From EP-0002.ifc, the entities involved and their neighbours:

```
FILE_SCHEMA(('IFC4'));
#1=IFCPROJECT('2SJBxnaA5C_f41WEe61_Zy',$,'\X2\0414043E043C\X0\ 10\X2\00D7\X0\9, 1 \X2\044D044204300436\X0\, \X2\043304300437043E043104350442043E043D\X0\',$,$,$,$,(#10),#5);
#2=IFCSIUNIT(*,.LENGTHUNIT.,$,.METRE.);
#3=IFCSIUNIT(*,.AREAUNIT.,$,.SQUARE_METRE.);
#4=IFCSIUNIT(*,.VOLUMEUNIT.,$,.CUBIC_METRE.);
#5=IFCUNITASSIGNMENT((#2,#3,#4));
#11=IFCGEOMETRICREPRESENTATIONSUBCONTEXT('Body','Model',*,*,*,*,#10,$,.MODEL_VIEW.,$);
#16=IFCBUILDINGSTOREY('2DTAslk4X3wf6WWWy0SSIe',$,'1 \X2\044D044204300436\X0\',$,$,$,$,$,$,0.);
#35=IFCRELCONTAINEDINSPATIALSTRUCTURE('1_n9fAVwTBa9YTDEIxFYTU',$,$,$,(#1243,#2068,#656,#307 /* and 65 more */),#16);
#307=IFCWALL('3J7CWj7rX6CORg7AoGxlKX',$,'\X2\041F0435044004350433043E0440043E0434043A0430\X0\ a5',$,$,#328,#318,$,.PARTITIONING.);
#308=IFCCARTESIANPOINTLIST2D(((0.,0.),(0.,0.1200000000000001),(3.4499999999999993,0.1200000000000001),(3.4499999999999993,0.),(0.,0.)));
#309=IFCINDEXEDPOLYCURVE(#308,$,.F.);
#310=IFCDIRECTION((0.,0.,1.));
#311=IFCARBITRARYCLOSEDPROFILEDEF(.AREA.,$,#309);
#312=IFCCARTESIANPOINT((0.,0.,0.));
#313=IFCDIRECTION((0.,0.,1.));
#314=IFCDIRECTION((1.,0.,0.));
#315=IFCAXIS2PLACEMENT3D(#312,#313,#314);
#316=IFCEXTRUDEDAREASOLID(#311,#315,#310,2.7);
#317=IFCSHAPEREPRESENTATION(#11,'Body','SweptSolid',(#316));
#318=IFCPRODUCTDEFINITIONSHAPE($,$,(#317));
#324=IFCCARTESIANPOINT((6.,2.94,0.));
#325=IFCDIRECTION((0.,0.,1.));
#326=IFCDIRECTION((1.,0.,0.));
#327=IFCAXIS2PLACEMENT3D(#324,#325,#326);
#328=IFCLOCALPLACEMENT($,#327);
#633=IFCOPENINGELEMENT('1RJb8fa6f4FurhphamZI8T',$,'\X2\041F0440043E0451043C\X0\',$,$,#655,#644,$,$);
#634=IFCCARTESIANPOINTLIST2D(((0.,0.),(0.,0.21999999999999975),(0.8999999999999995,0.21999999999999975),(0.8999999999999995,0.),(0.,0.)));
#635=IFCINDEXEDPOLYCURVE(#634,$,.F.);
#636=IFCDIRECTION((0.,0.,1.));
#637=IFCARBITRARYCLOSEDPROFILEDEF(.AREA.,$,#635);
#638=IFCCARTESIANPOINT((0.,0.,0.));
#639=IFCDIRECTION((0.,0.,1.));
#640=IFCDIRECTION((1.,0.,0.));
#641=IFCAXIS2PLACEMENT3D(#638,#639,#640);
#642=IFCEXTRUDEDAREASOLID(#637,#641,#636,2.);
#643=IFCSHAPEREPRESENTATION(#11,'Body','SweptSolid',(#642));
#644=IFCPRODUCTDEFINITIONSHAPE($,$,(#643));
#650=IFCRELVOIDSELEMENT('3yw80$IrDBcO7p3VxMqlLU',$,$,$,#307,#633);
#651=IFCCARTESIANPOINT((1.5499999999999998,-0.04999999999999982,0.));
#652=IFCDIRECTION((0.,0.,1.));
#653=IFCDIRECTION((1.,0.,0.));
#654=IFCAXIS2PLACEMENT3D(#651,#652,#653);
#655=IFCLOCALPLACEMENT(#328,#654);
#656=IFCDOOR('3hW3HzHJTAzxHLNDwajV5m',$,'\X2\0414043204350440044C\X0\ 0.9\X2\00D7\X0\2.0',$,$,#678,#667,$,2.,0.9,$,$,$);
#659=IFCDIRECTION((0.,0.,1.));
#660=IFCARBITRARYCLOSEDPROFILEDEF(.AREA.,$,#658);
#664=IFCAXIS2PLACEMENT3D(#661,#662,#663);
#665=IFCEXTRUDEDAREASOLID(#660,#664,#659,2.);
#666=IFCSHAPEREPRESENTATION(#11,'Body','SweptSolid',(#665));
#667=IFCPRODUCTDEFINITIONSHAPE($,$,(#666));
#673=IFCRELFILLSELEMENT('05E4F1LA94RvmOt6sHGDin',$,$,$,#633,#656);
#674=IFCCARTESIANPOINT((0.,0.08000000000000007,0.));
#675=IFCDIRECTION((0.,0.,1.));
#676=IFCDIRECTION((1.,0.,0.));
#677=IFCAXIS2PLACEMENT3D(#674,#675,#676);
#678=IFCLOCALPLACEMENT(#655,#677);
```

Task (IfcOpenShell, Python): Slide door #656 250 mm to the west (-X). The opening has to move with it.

```python
import ifcopenshell
import ifcopenshell.api.geometry
import ifcopenshell.util.placement

model = ifcopenshell.open("EP-0002.ifc")

door = model.by_guid("3hW3HzHJTAzxHLNDwajV5m")
opening = door.FillsVoids[0].RelatingOpeningElement
wall = opening.VoidsElements[0].RelatingBuildingElement

wall_matrix = ifcopenshell.util.placement.get_local_placement(wall.ObjectPlacement)
shift = wall_matrix[:3, 0] * -0.25
before = ifcopenshell.util.placement.get_local_placement(door.ObjectPlacement)[:3, 3].copy()

# The door is placed relative to its opening, so it follows when the opening moves.
matrix = ifcopenshell.util.placement.get_local_placement(opening.ObjectPlacement)
matrix[:3, 3] += shift
ifcopenshell.api.geometry.edit_object_placement(
    model, product=opening, matrix=matrix, is_si=False, should_transform_children=True
)

after = ifcopenshell.util.placement.get_local_placement(door.ObjectPlacement)[:3, 3]
print("door moved by", (after - before).round(3) + 0.0)

model.write("EP-0002_rev.ifc")
```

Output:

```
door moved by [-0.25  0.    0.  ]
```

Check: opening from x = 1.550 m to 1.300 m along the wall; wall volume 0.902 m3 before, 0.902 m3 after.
